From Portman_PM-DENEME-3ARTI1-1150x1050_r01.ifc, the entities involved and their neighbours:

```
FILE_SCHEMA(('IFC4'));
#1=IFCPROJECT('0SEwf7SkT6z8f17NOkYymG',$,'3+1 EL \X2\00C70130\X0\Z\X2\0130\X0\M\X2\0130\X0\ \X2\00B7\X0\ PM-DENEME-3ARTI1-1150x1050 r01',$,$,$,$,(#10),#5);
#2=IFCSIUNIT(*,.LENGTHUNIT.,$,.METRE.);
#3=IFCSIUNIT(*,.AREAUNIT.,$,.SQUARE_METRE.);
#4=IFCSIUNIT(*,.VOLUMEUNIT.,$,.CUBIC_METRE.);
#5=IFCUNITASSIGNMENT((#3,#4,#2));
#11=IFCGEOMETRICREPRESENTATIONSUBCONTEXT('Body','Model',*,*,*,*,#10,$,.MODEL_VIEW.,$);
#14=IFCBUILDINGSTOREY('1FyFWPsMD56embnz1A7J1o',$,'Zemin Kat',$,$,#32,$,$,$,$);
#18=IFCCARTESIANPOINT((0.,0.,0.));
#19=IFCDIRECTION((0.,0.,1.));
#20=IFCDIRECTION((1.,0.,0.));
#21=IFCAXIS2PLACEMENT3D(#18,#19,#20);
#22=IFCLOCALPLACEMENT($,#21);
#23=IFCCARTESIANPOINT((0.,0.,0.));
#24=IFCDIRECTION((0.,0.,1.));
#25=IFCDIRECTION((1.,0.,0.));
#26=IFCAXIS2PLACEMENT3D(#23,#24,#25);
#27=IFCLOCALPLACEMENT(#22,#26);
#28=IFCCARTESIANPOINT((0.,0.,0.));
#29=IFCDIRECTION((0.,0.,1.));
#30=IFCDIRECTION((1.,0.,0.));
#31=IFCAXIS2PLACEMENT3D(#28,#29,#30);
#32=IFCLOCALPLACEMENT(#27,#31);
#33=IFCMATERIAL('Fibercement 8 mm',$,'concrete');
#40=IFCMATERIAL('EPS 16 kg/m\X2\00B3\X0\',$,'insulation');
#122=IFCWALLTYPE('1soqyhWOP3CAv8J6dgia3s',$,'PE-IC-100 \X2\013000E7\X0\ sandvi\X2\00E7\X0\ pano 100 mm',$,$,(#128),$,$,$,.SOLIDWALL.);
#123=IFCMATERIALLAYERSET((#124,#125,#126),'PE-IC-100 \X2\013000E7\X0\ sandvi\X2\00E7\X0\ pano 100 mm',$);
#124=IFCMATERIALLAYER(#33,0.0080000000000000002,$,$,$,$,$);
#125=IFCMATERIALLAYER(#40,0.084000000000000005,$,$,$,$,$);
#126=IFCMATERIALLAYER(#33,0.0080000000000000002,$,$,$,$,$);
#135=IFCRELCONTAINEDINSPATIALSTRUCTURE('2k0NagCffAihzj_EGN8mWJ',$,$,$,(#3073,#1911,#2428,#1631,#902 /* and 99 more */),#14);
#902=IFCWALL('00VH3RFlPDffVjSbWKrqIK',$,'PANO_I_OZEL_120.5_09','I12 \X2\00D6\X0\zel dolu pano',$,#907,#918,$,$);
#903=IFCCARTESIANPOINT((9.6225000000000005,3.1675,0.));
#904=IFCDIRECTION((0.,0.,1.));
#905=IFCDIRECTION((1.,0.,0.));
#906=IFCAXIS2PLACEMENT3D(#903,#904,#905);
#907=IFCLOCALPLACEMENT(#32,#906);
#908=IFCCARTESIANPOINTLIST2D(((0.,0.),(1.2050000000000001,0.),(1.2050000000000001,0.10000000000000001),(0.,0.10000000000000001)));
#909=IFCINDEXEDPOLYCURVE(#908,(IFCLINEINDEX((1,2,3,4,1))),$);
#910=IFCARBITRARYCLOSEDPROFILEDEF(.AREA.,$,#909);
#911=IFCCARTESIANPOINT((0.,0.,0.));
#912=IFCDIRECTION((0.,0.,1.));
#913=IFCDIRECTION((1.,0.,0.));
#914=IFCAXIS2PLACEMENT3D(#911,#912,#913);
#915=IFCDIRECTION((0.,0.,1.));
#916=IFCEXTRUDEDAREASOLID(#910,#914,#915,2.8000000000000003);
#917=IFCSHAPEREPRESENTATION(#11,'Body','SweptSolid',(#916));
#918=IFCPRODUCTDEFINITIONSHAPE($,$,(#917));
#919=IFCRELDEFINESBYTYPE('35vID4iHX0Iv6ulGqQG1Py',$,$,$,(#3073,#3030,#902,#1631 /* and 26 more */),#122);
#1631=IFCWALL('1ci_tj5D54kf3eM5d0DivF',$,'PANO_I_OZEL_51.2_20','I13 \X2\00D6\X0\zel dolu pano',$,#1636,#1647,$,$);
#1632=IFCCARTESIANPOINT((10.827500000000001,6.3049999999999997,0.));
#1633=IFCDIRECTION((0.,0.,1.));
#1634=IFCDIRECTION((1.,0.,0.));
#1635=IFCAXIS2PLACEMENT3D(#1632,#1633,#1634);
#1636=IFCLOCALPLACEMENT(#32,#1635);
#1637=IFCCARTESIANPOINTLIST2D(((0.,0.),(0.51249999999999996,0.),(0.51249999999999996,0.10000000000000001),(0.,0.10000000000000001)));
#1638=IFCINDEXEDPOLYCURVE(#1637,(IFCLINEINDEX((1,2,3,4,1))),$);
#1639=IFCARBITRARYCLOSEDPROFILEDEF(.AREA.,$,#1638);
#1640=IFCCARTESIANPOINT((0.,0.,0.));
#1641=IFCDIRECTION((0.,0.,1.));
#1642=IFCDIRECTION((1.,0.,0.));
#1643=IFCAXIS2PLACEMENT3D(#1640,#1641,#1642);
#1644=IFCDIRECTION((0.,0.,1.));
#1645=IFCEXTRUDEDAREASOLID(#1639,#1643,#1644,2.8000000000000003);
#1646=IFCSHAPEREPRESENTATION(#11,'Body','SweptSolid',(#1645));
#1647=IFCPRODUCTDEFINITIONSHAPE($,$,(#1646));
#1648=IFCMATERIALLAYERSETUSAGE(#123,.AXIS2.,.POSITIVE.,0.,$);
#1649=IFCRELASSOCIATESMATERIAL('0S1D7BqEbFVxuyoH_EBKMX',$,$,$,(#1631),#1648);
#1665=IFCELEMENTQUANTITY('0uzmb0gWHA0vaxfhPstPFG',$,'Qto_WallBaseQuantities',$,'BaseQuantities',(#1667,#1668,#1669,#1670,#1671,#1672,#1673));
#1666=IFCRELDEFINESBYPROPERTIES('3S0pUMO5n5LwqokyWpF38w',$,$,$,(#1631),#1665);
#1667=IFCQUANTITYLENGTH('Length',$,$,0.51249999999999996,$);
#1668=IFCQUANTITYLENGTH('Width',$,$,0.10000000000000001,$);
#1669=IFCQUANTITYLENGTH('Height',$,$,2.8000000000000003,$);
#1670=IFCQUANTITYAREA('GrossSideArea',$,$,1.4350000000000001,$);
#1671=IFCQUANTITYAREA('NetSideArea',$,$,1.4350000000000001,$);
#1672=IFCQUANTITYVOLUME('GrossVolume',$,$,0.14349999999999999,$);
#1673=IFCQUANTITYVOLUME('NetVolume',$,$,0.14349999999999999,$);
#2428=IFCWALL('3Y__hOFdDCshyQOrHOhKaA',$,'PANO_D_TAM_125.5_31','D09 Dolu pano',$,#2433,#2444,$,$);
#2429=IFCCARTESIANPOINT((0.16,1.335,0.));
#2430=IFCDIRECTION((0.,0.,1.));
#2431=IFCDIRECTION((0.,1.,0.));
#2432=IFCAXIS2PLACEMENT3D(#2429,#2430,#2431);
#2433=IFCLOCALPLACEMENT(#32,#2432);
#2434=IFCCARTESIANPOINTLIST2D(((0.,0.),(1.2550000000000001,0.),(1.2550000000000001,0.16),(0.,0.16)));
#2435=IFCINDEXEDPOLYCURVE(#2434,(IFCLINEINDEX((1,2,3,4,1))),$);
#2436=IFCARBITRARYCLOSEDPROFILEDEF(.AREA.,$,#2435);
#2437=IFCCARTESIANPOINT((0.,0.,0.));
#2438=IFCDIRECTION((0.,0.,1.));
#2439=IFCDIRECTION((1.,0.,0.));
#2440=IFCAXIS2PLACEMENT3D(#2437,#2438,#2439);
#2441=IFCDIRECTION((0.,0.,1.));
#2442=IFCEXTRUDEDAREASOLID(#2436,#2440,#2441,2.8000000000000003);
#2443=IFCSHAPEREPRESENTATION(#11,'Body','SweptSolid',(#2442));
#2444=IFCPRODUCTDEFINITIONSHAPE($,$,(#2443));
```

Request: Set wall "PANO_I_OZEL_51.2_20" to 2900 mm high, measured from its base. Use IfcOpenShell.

```python
import ifcopenshell
import ifcopenshell.api.pset
import ifcopenshell.geom
import ifcopenshell.util.element
import ifcopenshell.util.representation
import ifcopenshell.util.shape
import ifcopenshell.util.unit

model = ifcopenshell.open("Portman_PM-DENEME-3ARTI1-1150x1050_r01.ifc")
unit_scale = ifcopenshell.util.unit.calculate_unit_scale(model)
area_scale = ifcopenshell.util.unit.calculate_unit_scale(model, "AREAUNIT")
volume_scale = ifcopenshell.util.unit.calculate_unit_scale(model, "VOLUMEUNIT")
settings = ifcopenshell.geom.settings()


def volume(element):
    """Net volume in cubic metres, openings subtracted."""
    shape = ifcopenshell.geom.create_shape(settings, element)
    return ifcopenshell.util.shape.get_volume(shape.geometry)


wall = model.by_guid("1ci_tj5D54kf3eM5d0DivF")
before = volume(wall)

body = ifcopenshell.util.representation.get_representation(wall, "Model", "Body")
solid = body.Items[0]
old_height = solid.Depth
solid.Depth = 2.9 / unit_scale
after = volume(wall)
thickness = 0.1  # wall thickness in metres

# Update the stored height, areas and volumes.
qto = model.by_id(ifcopenshell.util.element.get_pset(wall, "Qto_WallBaseQuantities", should_inherit=False)["id"])
ifcopenshell.api.pset.edit_qto(model, qto=qto, properties={
    "Height": solid.Depth,
    "GrossSideArea": ifcopenshell.util.element.get_pset(wall, "Qto_WallBaseQuantities", "GrossSideArea") * solid.Depth / old_height,
    "NetSideArea": after / thickness / area_scale,
    "GrossVolume": ifcopenshell.util.element.get_pset(wall, "Qto_WallBaseQuantities", "GrossVolume") * solid.Depth / old_height,
    "NetVolume": after / volume_scale,
})

print(f"height {old_height:g} -> {solid.Depth:g}, volume {before:.3f} -> {after:.3f} m3")

model.write("Portman_PM-DENEME-3ARTI1-1150x1050_r01-out.ifc")
```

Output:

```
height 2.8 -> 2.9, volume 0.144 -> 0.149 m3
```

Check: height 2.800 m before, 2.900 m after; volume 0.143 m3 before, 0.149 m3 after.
